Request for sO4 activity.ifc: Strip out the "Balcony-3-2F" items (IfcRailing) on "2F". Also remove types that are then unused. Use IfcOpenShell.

First a look at what the model holds.

```python
import ifcopenshell
import ifcopenshell.util.element

model = ifcopenshell.open("sO4 activity.ifc")
print(model.schema)
storey = next(s for s in model.by_type("IfcBuildingStorey") if s.Name == "2F")
railings = [e for e in ifcopenshell.util.element.get_decomposition(storey) if e.is_a("IfcRailing")]
seen = {}
for e in railings:
    element_type = ifcopenshell.util.element.get_type(e)
    name = element_type.Name if element_type not in (None, e) else None
    seen[name] = seen.get(name, 0) + 1
for name, count in sorted(seen.items(), key=str):
    print(count, "x", name)
```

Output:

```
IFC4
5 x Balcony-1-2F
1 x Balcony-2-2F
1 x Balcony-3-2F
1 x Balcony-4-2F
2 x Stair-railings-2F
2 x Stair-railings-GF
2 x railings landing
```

```python
import ifcopenshell
import ifcopenshell.api.root
import ifcopenshell.util.element

model = ifcopenshell.open("sO4 activity.ifc")

storey = next(s for s in model.by_type("IfcBuildingStorey") if s.Name == "2F")
railings = [e for e in ifcopenshell.util.element.get_decomposition(storey) if e.is_a("IfcRailing")]
targets = [e for e in railings if (t := ifcopenshell.util.element.get_type(e)) not in (None, e) and t.Name == "Balcony-3-2F"]
types = {ifcopenshell.util.element.get_type(e) for e in targets} - {None, *targets}

for e in targets:
    ifcopenshell.api.root.remove_product(model, product=e)
print(len(targets), "removed")

unused = [t for t in types if not ifcopenshell.util.element.get_types(t)]
for t in unused:
    ifcopenshell.api.root.remove_product(model, product=t)
print(len(unused), "unused types removed")

model.write("sO4 activity_updated.ifc")
```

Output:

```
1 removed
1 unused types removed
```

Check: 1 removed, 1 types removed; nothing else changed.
